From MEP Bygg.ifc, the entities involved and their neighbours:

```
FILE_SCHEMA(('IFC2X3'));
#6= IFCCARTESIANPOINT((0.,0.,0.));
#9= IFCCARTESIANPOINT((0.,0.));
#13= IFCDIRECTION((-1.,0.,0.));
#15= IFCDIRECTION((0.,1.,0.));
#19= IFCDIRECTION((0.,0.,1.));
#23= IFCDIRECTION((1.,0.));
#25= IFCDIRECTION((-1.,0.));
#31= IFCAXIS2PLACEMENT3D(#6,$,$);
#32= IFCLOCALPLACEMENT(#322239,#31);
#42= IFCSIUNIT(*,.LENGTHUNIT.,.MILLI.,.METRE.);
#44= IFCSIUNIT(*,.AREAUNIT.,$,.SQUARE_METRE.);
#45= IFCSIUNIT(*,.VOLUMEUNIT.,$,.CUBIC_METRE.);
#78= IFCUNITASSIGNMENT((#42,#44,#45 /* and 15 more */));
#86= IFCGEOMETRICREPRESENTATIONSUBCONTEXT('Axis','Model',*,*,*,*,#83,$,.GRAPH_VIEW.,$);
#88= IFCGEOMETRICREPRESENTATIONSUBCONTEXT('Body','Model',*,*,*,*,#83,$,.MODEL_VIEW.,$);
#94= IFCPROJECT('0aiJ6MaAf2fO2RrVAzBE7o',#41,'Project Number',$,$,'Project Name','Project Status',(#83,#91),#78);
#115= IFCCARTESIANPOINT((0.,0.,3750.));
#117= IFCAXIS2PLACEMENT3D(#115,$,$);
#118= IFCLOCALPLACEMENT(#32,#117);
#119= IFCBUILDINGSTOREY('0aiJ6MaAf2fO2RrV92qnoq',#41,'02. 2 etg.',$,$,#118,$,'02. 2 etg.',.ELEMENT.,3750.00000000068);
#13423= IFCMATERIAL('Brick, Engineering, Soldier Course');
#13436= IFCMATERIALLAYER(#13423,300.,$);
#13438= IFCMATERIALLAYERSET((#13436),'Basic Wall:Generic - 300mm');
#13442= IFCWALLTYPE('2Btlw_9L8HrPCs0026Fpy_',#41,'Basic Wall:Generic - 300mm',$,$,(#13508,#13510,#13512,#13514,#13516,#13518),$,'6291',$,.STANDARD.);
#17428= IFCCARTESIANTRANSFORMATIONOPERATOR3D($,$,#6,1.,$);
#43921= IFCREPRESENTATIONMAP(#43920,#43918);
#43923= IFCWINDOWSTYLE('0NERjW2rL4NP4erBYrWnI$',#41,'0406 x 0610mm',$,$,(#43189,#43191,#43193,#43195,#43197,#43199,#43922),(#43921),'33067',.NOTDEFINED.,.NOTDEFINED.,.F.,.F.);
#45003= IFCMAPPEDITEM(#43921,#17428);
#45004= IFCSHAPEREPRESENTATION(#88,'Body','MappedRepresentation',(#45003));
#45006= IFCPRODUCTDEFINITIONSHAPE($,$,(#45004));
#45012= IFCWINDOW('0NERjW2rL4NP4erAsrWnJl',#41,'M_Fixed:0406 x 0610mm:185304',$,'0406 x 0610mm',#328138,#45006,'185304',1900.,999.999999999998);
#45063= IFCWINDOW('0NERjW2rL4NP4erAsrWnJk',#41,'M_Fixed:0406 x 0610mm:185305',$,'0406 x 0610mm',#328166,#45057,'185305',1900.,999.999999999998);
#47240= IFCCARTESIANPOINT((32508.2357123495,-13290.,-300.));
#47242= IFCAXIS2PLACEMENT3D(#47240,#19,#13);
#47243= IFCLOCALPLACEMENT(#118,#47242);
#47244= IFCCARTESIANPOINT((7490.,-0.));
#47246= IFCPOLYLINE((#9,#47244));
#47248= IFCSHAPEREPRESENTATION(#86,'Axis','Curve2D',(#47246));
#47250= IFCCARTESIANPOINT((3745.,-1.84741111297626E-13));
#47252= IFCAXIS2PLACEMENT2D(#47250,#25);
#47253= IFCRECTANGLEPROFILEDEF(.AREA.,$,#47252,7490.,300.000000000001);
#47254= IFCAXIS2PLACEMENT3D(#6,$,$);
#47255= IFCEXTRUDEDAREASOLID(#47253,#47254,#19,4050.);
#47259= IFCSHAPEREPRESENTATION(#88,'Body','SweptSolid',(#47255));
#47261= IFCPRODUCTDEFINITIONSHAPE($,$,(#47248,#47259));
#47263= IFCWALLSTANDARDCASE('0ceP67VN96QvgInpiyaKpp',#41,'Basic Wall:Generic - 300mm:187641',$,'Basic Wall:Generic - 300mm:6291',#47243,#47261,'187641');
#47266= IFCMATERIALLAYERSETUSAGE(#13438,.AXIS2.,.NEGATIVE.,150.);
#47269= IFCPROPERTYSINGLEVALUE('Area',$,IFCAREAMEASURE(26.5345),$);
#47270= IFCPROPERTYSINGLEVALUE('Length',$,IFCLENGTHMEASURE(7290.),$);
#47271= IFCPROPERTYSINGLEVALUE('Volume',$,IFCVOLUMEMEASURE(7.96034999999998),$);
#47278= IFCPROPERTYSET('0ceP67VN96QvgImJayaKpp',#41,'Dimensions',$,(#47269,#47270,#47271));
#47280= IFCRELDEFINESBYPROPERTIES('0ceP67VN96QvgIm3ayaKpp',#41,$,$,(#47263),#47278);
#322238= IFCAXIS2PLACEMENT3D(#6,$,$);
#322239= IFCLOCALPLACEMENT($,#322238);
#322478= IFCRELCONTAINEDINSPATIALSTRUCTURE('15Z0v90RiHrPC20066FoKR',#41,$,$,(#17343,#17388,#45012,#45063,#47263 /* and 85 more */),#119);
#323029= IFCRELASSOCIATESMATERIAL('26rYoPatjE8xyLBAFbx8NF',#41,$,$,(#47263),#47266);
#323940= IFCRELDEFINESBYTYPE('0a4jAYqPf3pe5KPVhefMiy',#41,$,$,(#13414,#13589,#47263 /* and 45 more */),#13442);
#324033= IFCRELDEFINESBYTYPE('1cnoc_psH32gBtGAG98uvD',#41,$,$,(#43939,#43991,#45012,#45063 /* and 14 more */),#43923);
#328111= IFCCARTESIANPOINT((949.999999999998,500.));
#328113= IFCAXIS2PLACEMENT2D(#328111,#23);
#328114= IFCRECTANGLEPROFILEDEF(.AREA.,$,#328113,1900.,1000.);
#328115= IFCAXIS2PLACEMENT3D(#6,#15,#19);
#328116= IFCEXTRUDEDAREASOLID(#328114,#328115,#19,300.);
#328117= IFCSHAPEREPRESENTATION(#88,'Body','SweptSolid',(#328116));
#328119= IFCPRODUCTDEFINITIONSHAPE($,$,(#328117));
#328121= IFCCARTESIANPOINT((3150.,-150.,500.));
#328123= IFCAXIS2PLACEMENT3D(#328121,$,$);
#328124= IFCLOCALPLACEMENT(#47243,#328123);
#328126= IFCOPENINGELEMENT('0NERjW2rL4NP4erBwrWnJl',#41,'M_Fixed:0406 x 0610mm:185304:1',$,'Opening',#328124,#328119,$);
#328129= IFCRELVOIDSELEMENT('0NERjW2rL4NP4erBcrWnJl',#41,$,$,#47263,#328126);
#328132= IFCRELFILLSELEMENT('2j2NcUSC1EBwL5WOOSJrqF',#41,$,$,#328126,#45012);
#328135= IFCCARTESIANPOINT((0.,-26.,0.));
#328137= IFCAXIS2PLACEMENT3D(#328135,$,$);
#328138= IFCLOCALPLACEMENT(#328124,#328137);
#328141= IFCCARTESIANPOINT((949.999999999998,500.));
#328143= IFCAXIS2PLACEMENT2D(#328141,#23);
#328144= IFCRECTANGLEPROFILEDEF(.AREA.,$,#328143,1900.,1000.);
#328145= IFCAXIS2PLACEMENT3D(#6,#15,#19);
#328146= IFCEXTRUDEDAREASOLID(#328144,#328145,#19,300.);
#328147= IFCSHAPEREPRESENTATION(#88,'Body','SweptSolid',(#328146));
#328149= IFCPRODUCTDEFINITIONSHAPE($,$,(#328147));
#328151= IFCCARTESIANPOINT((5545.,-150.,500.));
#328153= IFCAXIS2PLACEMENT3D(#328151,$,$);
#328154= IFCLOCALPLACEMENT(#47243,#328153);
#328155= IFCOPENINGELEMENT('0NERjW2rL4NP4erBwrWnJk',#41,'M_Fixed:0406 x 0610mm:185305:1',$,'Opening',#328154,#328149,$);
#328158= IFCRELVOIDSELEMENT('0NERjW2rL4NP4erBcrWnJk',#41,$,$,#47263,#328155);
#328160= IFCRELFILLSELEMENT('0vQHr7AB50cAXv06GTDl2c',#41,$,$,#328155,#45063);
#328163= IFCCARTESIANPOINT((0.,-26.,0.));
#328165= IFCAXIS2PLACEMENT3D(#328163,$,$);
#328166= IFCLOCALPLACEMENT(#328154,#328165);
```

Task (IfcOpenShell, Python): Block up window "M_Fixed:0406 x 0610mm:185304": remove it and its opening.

```python
import ifcopenshell
import ifcopenshell.api.feature
import ifcopenshell.api.pset
import ifcopenshell.api.root
import ifcopenshell.geom
import ifcopenshell.util.element
import ifcopenshell.util.shape
import ifcopenshell.util.unit

model = ifcopenshell.open("MEP Bygg.ifc")
area_scale = ifcopenshell.util.unit.calculate_unit_scale(model, "AREAUNIT")
volume_scale = ifcopenshell.util.unit.calculate_unit_scale(model, "VOLUMEUNIT")
settings = ifcopenshell.geom.settings()


def volume(element):
    """Net volume in cubic metres, openings subtracted."""
    shape = ifcopenshell.geom.create_shape(settings, element)
    return ifcopenshell.util.shape.get_volume(shape.geometry)


window = model.by_guid("0NERjW2rL4NP4erAsrWnJl")
opening = window.FillsVoids[0].RelatingOpeningElement
wall = opening.VoidsElements[0].RelatingBuildingElement
before = volume(wall)

ifcopenshell.api.root.remove_product(model, product=window)
ifcopenshell.api.feature.remove_feature(model, feature=opening)

after = volume(wall)
thickness = 0.3  # wall thickness in metres

# Update the wall's stored quantities.
pset = model.by_id(ifcopenshell.util.element.get_pset(wall, "Dimensions", should_inherit=False)["id"])
ifcopenshell.api.pset.edit_pset(model, pset=pset, properties={
    "Area": model.create_entity("IfcAreaMeasure", after / thickness / area_scale),
    "Volume": model.create_entity("IfcVolumeMeasure", after / volume_scale),
})

print(f"wall volume {before:.3f} -> {after:.3f} m3")

model.write("MEP Bygg_updated.ifc")
```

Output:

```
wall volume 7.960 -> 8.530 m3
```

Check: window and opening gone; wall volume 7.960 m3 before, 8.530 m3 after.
